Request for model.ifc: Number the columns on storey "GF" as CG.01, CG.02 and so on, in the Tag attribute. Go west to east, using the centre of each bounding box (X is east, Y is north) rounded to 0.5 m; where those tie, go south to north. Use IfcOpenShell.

First a look at what the model holds.

```python
import ifcopenshell
import ifcopenshell.util.element
import ifcopenshell.util.placement

model = ifcopenshell.open("model.ifc")
print(model.schema)
storey = next(s for s in model.by_type("IfcBuildingStorey") if s.Name == "GF")
columns = [e for e in ifcopenshell.util.element.get_decomposition(storey) if e.is_a("IfcColumn")]
for e in sorted(columns, key=lambda e: e.id()):
    origin = ifcopenshell.util.placement.get_local_placement(e.ObjectPlacement)[:3, 3]
    print(e.id(), e.Tag, e.Name, origin.round(2) + 0.0, sep=" | ")
```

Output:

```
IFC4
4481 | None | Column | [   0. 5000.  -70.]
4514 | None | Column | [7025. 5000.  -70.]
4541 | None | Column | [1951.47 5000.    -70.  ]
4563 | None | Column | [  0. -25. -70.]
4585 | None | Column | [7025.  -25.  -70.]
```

```python
import ifcopenshell
import ifcopenshell.geom
import ifcopenshell.util.element
import ifcopenshell.util.shape

model = ifcopenshell.open("model.ifc")
settings = ifcopenshell.geom.settings()
settings.set("use-world-coords", True)


def centre(element):
    shape = ifcopenshell.geom.create_shape(settings, element)
    return ifcopenshell.util.shape.get_bbox_centroid(shape.geometry)


storey = next(s for s in model.by_type("IfcBuildingStorey") if s.Name == "GF")
columns = [e for e in ifcopenshell.util.element.get_decomposition(storey) if e.is_a("IfcColumn")]

# Insertion points can sit at a corner or the storey origin, so sort by the geometry (in metres).
centres = {e: centre(e) for e in columns}
columns.sort(key=lambda e: (round(centres[e][0] / 0.5), centres[e][1]))

for i, e in enumerate(columns, start=1):
    number = f"CG.{i:02d}"
    e.Tag = number
    print(e.id(), number)

model.write("model_rev.ifc")
```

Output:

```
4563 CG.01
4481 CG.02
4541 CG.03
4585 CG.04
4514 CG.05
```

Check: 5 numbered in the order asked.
